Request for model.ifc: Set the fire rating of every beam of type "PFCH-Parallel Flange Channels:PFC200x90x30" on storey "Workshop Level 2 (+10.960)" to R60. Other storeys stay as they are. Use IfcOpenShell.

First a look at what the model holds.

```python
import ifcopenshell
import ifcopenshell.util.element

model = ifcopenshell.open("model.ifc")
print(model.schema)
storey = next(s for s in model.by_type("IfcBuildingStorey") if s.Name == "Workshop Level 2 (+10.960)")
beams = [e for e in ifcopenshell.util.element.get_decomposition(storey) if e.is_a("IfcBeam")]
seen = {}
for e in beams:
    element_type = ifcopenshell.util.element.get_type(e)
    key = (element_type.Name if element_type != e and element_type else None, ifcopenshell.util.element.get_pset(e, "Pset_BeamCommon", "FireRating"))
    seen[key] = seen.get(key, 0) + 1
for (name, value), count in sorted(seen.items(), key=str):
    print(count, "x", name, "|", value)
```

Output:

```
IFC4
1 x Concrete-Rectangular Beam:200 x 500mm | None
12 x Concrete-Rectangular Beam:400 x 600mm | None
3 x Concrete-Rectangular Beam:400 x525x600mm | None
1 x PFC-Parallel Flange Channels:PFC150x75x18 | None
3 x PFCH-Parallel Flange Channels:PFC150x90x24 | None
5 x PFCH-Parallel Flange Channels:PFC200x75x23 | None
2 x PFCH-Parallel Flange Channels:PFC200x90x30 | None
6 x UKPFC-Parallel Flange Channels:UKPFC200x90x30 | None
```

```python
import ifcopenshell
import ifcopenshell.api.pset
import ifcopenshell.util.element

model = ifcopenshell.open("model.ifc")

storey = next(s for s in model.by_type("IfcBuildingStorey") if s.Name == "Workshop Level 2 (+10.960)")
beams = [e for e in ifcopenshell.util.element.get_decomposition(storey) if e.is_a("IfcBeam")]

count = 0
for e in beams:
    element_type = ifcopenshell.util.element.get_type(e)
    if element_type in (None, e) or element_type.Name != "PFCH-Parallel Flange Channels:PFC200x90x30":
        continue
    # add_pset returns the element's existing set when there is one.
    pset = ifcopenshell.api.pset.add_pset(model, product=e, name="Pset_BeamCommon")
    ifcopenshell.api.pset.edit_pset(model, pset=pset, properties={"FireRating": "R60"})
    count += 1

print(count, "beams updated")

model.write("model_rev.ifc")
```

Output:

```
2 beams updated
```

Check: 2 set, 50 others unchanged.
